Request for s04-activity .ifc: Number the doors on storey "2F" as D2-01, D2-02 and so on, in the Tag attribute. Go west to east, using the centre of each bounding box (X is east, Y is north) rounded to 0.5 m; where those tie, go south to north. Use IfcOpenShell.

First a look at what the model holds.

```python
import ifcopenshell
import ifcopenshell.util.element
import ifcopenshell.util.placement

model = ifcopenshell.open("s04-activity .ifc")
print(model.schema)
storey = next(s for s in model.by_type("IfcBuildingStorey") if s.Name == "2F")
doors = [e for e in ifcopenshell.util.element.get_decomposition(storey) if e.is_a("IfcDoor")]
for e in sorted(doors, key=lambda e: e.id()):
    origin = ifcopenshell.util.placement.get_local_placement(e.ObjectPlacement)[:3, 3]
    print(e.id(), e.Tag, e.Name, origin.round(2) + 0.0, sep=" | ")
```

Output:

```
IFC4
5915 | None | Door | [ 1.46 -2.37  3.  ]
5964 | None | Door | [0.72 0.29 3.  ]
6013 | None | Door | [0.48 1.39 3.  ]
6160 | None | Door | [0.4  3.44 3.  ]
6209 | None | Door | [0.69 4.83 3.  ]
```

```python
import ifcopenshell
import ifcopenshell.geom
import ifcopenshell.util.element
import ifcopenshell.util.shape

model = ifcopenshell.open("s04-activity .ifc")
settings = ifcopenshell.geom.settings()
settings.set("use-world-coords", True)


def centre(element):
    shape = ifcopenshell.geom.create_shape(settings, element)
    return ifcopenshell.util.shape.get_bbox_centroid(shape.geometry)


storey = next(s for s in model.by_type("IfcBuildingStorey") if s.Name == "2F")
doors = [e for e in ifcopenshell.util.element.get_decomposition(storey) if e.is_a("IfcDoor")]

# Insertion points can sit at a corner or the storey origin, so sort by the geometry (in metres).
centres = {e: centre(e) for e in doors}
doors.sort(key=lambda e: (round(centres[e][0] / 0.5), centres[e][1]))

for i, e in enumerate(doors, start=1):
    number = f"D2-{i:02d}"
    e.Tag = number
    print(e.id(), number)

model.write("s04-activity _edited.ifc")
```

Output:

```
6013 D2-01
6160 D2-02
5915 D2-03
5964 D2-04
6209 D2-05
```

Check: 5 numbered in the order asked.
